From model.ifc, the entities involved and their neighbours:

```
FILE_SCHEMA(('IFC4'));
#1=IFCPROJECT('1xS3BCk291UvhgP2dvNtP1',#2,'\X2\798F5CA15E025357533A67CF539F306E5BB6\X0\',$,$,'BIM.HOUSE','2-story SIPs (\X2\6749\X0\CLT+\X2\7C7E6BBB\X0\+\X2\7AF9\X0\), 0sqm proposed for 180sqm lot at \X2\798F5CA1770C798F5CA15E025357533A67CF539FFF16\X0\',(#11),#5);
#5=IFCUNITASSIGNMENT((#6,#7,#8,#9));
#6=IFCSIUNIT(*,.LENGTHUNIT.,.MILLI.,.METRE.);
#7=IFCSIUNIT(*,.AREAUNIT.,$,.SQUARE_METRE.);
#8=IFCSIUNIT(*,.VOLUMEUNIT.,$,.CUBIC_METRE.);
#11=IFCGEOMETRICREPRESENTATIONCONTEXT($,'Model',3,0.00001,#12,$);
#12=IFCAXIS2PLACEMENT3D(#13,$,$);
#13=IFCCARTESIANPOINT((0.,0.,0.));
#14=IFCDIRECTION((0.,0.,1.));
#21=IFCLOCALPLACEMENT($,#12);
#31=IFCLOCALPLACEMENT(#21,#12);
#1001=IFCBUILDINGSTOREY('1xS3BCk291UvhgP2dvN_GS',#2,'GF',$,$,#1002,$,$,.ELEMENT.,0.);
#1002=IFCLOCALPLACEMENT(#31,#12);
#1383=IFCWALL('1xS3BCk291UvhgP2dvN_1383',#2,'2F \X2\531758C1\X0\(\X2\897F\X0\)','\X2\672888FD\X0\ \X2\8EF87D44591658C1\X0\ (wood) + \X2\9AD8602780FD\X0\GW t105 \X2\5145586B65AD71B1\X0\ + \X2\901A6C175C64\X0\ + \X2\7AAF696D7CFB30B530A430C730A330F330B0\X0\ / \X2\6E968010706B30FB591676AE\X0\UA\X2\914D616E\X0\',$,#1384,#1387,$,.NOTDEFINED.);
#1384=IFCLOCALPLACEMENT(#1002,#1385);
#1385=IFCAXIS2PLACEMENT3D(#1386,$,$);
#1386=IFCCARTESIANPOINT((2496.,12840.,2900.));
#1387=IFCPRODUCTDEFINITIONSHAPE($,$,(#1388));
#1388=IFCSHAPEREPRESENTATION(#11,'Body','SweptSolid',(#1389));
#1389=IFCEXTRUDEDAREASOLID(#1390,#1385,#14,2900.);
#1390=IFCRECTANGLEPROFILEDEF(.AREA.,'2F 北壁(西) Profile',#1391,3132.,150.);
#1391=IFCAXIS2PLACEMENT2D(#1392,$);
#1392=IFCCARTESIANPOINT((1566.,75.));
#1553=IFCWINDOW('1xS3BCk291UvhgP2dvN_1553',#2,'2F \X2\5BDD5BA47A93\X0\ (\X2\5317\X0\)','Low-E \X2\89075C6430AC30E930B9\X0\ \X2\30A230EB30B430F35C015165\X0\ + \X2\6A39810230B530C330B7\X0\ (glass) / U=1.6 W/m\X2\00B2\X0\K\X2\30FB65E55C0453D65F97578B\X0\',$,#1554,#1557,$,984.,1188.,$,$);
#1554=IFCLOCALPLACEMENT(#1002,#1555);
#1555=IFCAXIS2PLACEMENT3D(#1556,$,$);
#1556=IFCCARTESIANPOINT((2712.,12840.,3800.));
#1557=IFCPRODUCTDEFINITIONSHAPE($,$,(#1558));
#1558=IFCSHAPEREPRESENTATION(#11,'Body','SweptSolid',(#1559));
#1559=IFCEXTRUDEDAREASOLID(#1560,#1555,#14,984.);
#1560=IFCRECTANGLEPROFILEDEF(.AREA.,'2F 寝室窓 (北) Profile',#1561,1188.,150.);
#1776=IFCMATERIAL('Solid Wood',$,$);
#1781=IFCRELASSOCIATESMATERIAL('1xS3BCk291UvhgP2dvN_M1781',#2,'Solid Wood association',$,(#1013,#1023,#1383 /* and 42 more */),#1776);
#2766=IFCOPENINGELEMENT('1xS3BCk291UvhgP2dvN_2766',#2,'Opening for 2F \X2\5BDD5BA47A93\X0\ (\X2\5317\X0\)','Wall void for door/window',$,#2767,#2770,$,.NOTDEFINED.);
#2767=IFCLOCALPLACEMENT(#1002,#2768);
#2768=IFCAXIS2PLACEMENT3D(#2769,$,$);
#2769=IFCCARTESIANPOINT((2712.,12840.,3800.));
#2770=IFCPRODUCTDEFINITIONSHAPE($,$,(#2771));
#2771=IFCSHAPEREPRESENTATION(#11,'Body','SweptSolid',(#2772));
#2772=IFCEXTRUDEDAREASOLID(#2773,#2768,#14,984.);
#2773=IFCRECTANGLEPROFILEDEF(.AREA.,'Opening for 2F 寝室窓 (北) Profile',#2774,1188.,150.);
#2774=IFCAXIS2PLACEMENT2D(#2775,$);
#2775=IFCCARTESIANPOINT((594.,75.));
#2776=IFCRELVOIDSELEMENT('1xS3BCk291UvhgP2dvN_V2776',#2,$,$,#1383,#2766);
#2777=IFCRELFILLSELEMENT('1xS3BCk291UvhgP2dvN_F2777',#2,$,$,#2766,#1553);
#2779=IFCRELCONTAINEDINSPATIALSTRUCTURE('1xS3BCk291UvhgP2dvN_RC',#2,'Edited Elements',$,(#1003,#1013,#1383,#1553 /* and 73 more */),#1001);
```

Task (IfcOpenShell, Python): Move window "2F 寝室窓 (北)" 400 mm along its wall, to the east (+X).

```python
import ifcopenshell
import ifcopenshell.api.geometry
import ifcopenshell.util.placement
import ifcopenshell.util.unit

model = ifcopenshell.open("model.ifc")
unit_scale = ifcopenshell.util.unit.calculate_unit_scale(model)

window = model.by_id(1553)
opening = window.FillsVoids[0].RelatingOpeningElement
wall = opening.VoidsElements[0].RelatingBuildingElement

wall_matrix = ifcopenshell.util.placement.get_local_placement(wall.ObjectPlacement)
shift = wall_matrix[:3, 0] * 0.4 / unit_scale
before = ifcopenshell.util.placement.get_local_placement(window.ObjectPlacement)[:3, 3].copy()

# The window is not placed relative to its opening, so move both.
for product in (opening, window):
    matrix = ifcopenshell.util.placement.get_local_placement(product.ObjectPlacement)
    matrix[:3, 3] += shift
    ifcopenshell.api.geometry.edit_object_placement(model, product=product, matrix=matrix, is_si=False)

after = ifcopenshell.util.placement.get_local_placement(window.ObjectPlacement)[:3, 3]
print("window moved by", (after - before).round(3) + 0.0)

model.write("model_updated.ifc")
```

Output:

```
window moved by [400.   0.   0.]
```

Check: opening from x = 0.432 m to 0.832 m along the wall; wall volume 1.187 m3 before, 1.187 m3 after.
